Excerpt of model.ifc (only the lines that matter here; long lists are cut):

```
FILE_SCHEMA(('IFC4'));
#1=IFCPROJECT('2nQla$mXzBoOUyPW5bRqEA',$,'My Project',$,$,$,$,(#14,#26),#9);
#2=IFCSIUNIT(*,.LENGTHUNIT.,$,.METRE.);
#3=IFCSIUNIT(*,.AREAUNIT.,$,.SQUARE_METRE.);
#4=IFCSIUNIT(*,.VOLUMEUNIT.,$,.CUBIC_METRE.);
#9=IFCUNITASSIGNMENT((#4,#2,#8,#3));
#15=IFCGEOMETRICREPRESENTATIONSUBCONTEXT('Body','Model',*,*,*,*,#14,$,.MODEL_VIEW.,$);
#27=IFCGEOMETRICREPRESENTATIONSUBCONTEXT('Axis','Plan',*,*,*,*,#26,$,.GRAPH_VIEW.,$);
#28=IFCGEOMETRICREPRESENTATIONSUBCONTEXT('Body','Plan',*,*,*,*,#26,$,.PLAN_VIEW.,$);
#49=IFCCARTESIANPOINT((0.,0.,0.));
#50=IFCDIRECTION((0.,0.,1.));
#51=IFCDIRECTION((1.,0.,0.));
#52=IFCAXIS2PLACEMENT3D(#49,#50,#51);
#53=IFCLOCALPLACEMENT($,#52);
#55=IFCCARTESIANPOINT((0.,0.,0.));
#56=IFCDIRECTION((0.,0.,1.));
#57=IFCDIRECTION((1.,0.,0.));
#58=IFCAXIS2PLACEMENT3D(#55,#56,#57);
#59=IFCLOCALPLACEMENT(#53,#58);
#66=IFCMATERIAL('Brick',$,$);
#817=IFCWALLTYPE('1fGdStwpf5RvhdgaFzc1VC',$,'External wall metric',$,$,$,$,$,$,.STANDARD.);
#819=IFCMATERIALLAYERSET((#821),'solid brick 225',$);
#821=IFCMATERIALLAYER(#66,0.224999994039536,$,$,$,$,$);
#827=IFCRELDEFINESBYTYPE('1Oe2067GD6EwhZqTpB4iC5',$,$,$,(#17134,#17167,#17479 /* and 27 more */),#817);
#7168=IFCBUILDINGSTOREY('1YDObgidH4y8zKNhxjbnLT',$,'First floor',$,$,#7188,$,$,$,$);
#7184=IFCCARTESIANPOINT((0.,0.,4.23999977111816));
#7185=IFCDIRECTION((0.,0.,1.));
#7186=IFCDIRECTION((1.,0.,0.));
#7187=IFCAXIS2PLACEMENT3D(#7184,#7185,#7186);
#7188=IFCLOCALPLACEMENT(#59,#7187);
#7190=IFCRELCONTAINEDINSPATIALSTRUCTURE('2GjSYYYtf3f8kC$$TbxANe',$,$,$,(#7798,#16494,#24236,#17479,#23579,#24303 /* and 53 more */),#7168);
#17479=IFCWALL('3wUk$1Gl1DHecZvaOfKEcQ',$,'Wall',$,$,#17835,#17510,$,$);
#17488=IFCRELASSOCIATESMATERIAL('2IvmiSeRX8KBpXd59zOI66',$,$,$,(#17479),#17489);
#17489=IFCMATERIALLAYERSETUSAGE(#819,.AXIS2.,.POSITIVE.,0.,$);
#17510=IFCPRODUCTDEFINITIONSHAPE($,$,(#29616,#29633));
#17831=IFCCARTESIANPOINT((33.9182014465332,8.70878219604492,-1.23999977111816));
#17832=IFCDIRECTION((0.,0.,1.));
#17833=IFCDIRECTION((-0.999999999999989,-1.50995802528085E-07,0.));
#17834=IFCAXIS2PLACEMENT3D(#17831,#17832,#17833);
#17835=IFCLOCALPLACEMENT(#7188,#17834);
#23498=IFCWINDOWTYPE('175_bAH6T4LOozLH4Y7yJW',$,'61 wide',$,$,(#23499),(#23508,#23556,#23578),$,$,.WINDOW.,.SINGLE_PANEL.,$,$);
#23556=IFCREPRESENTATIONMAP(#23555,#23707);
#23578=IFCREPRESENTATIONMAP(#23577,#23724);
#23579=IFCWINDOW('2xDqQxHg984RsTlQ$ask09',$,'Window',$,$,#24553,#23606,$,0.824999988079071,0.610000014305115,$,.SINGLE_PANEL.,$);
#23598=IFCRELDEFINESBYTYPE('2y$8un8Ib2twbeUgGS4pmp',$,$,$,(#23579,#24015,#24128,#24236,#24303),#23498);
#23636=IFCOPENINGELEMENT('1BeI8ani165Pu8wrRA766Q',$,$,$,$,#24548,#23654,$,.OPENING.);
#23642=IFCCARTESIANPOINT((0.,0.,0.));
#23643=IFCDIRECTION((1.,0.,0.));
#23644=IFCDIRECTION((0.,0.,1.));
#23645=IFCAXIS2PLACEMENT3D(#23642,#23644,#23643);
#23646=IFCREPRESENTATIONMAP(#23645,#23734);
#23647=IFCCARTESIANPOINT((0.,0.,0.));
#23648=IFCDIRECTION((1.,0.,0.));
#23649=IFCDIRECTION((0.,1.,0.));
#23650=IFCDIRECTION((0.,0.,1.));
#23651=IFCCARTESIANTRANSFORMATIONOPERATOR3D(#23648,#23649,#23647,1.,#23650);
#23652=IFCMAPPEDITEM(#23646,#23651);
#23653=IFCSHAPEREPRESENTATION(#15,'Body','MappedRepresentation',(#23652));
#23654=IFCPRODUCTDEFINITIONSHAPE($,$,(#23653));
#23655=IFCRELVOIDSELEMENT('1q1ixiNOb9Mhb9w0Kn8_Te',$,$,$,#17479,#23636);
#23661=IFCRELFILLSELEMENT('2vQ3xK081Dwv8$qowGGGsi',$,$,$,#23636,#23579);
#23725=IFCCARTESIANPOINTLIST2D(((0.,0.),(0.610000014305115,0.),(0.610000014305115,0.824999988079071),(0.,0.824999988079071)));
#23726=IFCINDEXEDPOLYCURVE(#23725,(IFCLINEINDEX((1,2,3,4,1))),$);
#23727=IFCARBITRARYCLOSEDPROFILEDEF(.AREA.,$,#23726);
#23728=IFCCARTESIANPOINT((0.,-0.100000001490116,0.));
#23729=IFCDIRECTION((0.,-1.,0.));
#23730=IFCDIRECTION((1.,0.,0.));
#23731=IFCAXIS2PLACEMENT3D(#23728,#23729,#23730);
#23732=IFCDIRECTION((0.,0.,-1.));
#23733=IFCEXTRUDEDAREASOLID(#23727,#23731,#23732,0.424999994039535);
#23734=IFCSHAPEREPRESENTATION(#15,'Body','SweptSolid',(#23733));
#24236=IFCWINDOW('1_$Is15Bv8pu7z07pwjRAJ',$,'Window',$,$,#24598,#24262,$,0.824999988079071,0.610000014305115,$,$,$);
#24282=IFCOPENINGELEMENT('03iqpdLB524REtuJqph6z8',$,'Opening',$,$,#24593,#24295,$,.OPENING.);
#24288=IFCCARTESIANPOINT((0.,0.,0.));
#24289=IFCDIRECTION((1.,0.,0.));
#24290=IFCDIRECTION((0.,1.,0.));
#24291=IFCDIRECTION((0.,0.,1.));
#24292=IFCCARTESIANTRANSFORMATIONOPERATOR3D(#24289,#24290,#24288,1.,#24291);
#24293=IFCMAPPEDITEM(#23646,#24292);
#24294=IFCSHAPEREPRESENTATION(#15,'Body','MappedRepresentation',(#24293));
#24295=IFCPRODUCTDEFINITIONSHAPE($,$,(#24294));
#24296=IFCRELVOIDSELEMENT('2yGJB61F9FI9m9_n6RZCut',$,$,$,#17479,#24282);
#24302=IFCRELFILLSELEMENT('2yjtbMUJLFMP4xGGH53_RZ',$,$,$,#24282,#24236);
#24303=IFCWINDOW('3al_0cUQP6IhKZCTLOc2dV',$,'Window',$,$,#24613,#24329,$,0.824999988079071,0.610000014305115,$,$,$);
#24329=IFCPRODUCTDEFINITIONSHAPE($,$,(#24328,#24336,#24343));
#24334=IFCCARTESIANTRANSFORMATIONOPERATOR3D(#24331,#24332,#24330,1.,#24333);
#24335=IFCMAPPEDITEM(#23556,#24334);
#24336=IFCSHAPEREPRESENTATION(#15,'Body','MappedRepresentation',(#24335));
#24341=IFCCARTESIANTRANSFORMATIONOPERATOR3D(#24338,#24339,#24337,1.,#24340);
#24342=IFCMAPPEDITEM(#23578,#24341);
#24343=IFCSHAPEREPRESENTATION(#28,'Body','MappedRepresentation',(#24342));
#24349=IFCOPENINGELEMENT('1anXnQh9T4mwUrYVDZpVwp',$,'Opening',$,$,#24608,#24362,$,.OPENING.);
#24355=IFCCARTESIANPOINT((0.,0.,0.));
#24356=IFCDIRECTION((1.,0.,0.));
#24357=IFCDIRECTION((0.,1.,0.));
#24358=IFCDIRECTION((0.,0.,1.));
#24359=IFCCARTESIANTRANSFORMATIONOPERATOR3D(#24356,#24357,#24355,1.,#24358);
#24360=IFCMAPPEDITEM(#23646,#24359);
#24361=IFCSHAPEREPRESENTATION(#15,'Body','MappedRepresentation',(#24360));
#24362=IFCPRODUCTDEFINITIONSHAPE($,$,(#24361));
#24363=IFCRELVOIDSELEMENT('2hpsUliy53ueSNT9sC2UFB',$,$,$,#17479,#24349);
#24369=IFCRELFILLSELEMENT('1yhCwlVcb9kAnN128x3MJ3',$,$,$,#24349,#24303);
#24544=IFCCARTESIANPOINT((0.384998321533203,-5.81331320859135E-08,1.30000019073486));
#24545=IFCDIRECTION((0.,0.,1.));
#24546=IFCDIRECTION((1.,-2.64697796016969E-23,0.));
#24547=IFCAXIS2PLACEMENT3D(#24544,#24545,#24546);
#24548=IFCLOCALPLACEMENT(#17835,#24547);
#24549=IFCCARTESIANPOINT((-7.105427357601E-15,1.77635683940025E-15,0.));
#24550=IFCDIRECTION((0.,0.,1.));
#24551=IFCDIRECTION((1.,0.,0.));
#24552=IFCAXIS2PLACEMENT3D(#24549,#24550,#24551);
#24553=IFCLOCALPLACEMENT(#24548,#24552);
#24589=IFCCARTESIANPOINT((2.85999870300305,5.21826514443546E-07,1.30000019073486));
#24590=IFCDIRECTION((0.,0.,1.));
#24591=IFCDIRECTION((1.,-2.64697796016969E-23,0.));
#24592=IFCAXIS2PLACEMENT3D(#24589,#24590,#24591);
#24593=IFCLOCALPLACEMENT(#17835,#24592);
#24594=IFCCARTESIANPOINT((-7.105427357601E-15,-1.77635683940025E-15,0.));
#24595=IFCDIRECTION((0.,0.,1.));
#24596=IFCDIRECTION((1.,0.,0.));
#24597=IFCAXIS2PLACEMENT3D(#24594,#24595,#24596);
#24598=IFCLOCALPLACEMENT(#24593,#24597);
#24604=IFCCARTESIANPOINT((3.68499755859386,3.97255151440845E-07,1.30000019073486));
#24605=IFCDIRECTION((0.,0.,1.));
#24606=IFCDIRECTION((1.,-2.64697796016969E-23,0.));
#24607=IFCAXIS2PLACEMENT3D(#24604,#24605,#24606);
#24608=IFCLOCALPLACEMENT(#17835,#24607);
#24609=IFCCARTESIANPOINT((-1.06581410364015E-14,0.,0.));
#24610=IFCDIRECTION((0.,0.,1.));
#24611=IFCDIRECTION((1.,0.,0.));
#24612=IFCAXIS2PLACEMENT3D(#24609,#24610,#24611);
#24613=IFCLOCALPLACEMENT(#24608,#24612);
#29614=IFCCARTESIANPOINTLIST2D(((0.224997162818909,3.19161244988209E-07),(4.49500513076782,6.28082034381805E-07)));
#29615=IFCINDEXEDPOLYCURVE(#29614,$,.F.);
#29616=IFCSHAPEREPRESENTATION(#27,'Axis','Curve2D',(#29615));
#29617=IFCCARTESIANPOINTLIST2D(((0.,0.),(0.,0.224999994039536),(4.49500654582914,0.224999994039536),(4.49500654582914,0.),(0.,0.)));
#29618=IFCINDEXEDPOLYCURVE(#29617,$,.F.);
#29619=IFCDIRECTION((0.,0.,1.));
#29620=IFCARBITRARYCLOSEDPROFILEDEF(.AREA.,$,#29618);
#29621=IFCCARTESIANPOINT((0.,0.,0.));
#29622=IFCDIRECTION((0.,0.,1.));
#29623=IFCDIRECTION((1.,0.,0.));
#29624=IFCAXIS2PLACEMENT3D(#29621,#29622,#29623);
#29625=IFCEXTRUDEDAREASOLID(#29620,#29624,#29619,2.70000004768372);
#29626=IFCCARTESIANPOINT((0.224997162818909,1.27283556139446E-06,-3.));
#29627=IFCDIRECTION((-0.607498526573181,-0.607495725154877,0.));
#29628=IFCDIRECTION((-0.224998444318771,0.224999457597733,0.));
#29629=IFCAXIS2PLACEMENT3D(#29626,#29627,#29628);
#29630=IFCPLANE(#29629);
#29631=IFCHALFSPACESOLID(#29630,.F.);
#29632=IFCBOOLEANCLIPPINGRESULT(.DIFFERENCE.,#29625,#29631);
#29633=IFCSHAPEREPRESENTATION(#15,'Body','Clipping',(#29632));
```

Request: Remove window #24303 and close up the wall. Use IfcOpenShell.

```python
import ifcopenshell
import ifcopenshell.api.feature
import ifcopenshell.api.root
import ifcopenshell.geom
import ifcopenshell.util.shape

model = ifcopenshell.open("model.ifc")
settings = ifcopenshell.geom.settings()


def volume(element):
    """Net volume in cubic metres, openings subtracted."""
    shape = ifcopenshell.geom.create_shape(settings, element)
    return ifcopenshell.util.shape.get_volume(shape.geometry)


window = model.by_guid("3al_0cUQP6IhKZCTLOc2dV")
opening = window.FillsVoids[0].RelatingOpeningElement
wall = opening.VoidsElements[0].RelatingBuildingElement
before = volume(wall)

ifcopenshell.api.root.remove_product(model, product=window)
ifcopenshell.api.feature.remove_feature(model, feature=opening)

after = volume(wall)

print(f"wall volume {before:.3f} -> {after:.3f} m3")

model.write("model_updated.ifc")
```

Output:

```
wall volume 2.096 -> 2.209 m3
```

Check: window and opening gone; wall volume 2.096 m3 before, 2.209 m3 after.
